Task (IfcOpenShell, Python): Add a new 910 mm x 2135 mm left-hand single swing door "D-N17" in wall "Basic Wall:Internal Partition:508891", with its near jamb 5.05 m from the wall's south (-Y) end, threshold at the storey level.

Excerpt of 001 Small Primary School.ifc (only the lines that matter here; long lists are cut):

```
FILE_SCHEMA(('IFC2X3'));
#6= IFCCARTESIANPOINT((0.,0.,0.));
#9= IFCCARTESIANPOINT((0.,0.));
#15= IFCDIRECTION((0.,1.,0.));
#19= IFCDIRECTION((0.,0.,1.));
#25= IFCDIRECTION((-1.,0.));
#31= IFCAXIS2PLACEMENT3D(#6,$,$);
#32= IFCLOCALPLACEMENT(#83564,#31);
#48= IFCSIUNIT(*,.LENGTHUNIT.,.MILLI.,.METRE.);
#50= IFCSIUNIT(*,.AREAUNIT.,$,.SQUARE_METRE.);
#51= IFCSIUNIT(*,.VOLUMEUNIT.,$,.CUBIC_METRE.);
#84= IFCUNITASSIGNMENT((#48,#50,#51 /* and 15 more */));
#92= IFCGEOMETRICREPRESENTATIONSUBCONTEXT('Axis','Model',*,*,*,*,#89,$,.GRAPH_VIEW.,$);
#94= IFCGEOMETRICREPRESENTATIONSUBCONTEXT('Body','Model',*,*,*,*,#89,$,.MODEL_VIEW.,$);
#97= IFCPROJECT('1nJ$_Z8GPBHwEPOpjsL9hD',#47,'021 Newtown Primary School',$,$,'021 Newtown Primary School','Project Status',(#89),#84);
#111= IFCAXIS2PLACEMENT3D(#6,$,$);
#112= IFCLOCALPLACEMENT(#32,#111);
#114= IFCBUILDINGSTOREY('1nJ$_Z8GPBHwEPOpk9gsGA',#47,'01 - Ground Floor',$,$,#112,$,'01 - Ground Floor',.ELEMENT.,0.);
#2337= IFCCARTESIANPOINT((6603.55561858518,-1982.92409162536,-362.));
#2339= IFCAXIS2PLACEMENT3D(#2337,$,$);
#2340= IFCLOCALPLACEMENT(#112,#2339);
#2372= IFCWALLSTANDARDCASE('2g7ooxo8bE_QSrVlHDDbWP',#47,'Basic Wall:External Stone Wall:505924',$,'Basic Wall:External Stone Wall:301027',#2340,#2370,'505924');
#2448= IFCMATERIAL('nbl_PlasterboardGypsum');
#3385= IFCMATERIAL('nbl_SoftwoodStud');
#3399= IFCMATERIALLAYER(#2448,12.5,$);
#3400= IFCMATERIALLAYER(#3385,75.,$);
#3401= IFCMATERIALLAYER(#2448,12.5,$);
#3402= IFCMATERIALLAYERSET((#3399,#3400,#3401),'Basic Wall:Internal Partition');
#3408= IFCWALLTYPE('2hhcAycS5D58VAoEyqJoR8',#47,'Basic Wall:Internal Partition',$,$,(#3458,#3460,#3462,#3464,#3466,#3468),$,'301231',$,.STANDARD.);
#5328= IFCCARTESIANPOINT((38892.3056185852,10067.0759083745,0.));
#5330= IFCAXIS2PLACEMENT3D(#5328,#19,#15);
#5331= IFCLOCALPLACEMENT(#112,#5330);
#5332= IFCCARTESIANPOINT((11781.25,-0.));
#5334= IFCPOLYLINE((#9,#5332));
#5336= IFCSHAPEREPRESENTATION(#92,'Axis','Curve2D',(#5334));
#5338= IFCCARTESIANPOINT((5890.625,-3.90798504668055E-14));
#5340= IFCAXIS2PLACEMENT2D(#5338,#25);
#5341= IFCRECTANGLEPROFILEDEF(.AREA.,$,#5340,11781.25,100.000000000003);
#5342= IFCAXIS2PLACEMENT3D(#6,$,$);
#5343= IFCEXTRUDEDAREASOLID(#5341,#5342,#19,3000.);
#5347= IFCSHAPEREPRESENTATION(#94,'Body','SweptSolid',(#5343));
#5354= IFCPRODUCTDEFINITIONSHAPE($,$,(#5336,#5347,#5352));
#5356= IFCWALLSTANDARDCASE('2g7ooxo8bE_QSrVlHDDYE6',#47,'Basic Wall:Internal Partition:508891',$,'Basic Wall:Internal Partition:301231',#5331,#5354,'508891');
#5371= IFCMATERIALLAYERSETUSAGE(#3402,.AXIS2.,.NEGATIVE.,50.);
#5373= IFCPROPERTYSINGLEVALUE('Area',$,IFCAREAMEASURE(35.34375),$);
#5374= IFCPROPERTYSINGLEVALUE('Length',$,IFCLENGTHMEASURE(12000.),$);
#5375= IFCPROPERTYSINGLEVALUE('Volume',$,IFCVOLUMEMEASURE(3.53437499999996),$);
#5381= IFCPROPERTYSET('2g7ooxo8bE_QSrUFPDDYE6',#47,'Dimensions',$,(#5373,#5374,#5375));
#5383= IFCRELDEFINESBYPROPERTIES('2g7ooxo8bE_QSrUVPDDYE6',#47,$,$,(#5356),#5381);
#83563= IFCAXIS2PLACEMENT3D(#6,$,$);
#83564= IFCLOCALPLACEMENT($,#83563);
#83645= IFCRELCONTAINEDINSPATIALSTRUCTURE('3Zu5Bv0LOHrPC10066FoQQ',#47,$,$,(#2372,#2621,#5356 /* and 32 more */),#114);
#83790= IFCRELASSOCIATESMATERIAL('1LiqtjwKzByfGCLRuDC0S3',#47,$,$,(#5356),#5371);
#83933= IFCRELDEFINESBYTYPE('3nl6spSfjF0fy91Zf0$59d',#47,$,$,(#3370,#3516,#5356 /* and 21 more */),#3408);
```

```python
import numpy as np
import ifcopenshell
import ifcopenshell.api.feature
import ifcopenshell.api.geometry
import ifcopenshell.api.pset
import ifcopenshell.api.root
import ifcopenshell.api.spatial
import ifcopenshell.api.type
import ifcopenshell.geom
import ifcopenshell.util.element
import ifcopenshell.util.placement
import ifcopenshell.util.representation
import ifcopenshell.util.shape
import ifcopenshell.util.unit

model = ifcopenshell.open("001 Small Primary School.ifc")
unit_scale = ifcopenshell.util.unit.calculate_unit_scale(model)
area_scale = ifcopenshell.util.unit.calculate_unit_scale(model, "AREAUNIT")
volume_scale = ifcopenshell.util.unit.calculate_unit_scale(model, "VOLUMEUNIT")
settings = ifcopenshell.geom.settings()


def volume(element):
    """Net volume in cubic metres, openings subtracted."""
    shape = ifcopenshell.geom.create_shape(settings, element)
    return ifcopenshell.util.shape.get_volume(shape.geometry)


wall = model.by_id(5356)
storey = ifcopenshell.util.element.get_container(wall, ifc_class="IfcBuildingStorey")
context = ifcopenshell.util.representation.get_context(model, "Model", "Body", "MODEL_VIEW")
before = volume(wall)

width, height, from_end, sill = 0.91, 2.135, 5.05, 0.0  # metres

# The wall runs along its own X axis, and the end named is its -X end.
wall_shape = ifcopenshell.geom.create_shape(settings, wall)
x, y, z = ifcopenshell.util.shape.get_vertices(wall_shape.geometry).T
start = x.min() + from_end
face, thickness = float(y.min()), float(y.max() - y.min())
wall_matrix = ifcopenshell.util.placement.get_local_placement(wall.ObjectPlacement)
level = ifcopenshell.util.placement.get_local_placement(storey.ObjectPlacement)[2, 3]


def in_wall(x, y):
    """Placement at x, y metres in the wall's axes, at sill height."""
    matrix = wall_matrix.copy()
    matrix[:, 3] = wall_matrix @ np.array([x / unit_scale, y / unit_scale, 0.0, 1.0])
    matrix[2, 3] = level + sill / unit_scale
    return matrix


# Opening: a box that overshoots both wall faces by 50 mm.
opening = ifcopenshell.api.root.create_entity(model, ifc_class="IfcOpeningElement")
box = ifcopenshell.api.geometry.add_wall_representation(
    model, context=context, length=width, height=height, thickness=thickness + 0.1
)
ifcopenshell.api.geometry.assign_representation(model, product=opening, representation=box)
ifcopenshell.api.geometry.edit_object_placement(model, product=opening, matrix=in_wall(start, face - 0.05), is_si=False)
ifcopenshell.api.feature.add_feature(model, feature=opening, element=wall)

door = ifcopenshell.api.root.create_entity(model, ifc_class="IfcDoor", name="D-N17")
door.OverallWidth, door.OverallHeight = width / unit_scale, height / unit_scale
body = ifcopenshell.api.geometry.add_door_representation(
    model,
    context=context,
    overall_width=door.OverallWidth,
    overall_height=door.OverallHeight,
    operation_type="SINGLE_SWING_LEFT",
    lining_properties={"LiningDepth": thickness / unit_scale, "ThresholdDepth": thickness / unit_scale},
)
ifcopenshell.api.geometry.assign_representation(model, product=door, representation=body)
ifcopenshell.api.spatial.assign_container(model, products=[door], relating_structure=storey)
fills = ifcopenshell.api.feature.add_filling(model, opening=opening, element=door)
fills.OwnerHistory = door.OwnerHistory  # required in IFC2X3

# IFC2X3 keeps the operation on the door style.
style = ifcopenshell.api.root.create_entity(model, ifc_class="IfcDoorStyle", name="D-N17")
style.OperationType, style.ConstructionType = "SINGLE_SWING_LEFT", "NOTDEFINED"
style.ParameterTakesPrecedence = style.Sizeable = False
ifcopenshell.api.type.assign_type(model, related_objects=[door], relating_type=style)

# The lining spans the wall, so the door starts at the wall face.
ifcopenshell.api.geometry.edit_object_placement(model, product=door, matrix=in_wall(start, face), is_si=False)

after = volume(wall)

# Update the wall's stored quantities.
pset = model.by_id(ifcopenshell.util.element.get_pset(wall, "Dimensions", should_inherit=False)["id"])
ifcopenshell.api.pset.edit_pset(model, pset=pset, properties={
    "Area": model.create_entity("IfcAreaMeasure", after / thickness / area_scale),
    "Volume": model.create_entity("IfcVolumeMeasure", after / volume_scale),
})

print(f"wall volume {before:.3f} -> {after:.3f} m3")

model.write("001 Small Primary School_rev.ifc")
```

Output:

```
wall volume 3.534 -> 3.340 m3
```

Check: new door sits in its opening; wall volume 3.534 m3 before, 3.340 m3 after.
